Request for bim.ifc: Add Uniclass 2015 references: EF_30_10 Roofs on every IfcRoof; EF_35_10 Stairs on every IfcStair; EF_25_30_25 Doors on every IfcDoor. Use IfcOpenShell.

First a look at what the model holds.

```python
import ifcopenshell

model = ifcopenshell.open("bim.ifc")
print(model.schema)
print("classifications:", [c.Name for c in model.by_type("IfcClassification")])
for ifc_class in ("IfcDoor", "IfcRoof", "IfcStair", "IfcWall", "IfcWindow"):
    print(ifc_class, len(model.by_type(ifc_class)))
```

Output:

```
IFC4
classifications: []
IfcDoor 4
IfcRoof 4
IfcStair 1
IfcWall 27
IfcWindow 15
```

```python
import ifcopenshell
import ifcopenshell.api.classification

model = ifcopenshell.open("bim.ifc")

system = ifcopenshell.api.classification.add_classification(model, classification="Uniclass 2015")

codes = {
    "IfcRoof": ("EF_30_10", "Roofs"),
    "IfcStair": ("EF_35_10", "Stairs"),
    "IfcDoor": ("EF_25_30_25", "Doors"),
}
for ifc_class, (code, name) in codes.items():
    products = model.by_type(ifc_class)
    ifcopenshell.api.classification.add_reference(
        model, products=products, classification=system, identification=code, name=name
    )
    print(code, len(products))

model.write("bim_edited.ifc")
```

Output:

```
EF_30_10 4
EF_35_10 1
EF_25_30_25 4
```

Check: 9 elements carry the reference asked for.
